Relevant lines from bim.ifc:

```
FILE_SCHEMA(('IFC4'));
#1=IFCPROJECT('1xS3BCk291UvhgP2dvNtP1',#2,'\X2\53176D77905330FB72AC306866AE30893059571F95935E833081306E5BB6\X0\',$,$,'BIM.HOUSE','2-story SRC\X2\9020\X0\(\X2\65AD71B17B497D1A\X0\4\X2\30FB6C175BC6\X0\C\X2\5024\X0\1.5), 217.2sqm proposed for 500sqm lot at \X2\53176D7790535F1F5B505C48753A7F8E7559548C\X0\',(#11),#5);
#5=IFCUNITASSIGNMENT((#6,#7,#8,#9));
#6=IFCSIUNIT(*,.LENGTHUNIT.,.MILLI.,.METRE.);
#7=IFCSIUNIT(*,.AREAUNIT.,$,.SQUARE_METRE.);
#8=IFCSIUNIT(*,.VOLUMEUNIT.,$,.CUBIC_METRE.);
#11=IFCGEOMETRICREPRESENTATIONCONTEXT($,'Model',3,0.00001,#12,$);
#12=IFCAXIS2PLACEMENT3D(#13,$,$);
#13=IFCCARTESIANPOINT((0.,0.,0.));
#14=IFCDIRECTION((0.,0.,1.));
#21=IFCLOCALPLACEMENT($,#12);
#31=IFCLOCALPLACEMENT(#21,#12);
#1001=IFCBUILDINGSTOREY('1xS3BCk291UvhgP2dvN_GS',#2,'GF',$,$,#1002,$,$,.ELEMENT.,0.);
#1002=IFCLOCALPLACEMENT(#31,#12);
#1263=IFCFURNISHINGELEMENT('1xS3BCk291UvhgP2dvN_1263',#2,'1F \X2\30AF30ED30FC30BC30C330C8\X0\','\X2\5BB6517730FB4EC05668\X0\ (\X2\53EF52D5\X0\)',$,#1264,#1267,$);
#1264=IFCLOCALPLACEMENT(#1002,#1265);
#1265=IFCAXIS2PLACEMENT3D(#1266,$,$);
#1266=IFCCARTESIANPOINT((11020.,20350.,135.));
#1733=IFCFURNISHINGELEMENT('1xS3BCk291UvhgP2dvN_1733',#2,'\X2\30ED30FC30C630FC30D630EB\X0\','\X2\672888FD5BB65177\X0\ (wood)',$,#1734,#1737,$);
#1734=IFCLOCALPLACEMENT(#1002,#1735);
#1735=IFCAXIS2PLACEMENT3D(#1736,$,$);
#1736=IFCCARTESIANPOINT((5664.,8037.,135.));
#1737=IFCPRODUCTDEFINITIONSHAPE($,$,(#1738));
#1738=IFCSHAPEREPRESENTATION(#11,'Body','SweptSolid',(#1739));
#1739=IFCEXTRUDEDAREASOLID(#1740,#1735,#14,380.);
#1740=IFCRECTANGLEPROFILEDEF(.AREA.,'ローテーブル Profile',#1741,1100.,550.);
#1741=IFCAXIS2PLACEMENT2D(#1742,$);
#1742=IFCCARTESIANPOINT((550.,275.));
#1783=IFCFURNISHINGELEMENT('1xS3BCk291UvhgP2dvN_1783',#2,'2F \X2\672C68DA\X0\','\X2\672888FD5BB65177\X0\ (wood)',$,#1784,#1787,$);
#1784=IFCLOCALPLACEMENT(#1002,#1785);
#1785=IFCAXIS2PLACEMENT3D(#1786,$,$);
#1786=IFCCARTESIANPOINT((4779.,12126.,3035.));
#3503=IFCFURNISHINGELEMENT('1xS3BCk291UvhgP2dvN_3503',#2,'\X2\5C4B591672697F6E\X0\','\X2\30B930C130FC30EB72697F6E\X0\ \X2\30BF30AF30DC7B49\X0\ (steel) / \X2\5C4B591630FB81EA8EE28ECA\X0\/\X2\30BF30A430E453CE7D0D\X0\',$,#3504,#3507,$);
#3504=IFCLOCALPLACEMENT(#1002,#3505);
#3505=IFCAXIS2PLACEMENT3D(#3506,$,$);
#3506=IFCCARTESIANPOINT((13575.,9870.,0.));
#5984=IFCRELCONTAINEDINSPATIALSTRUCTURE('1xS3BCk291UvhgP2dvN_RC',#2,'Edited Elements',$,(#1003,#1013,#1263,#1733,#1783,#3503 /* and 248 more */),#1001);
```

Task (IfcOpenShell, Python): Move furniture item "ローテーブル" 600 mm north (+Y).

```python
import ifcopenshell
import ifcopenshell.api.geometry
import ifcopenshell.util.placement

model = ifcopenshell.open("bim.ifc")

item = model.by_guid("1xS3BCk291UvhgP2dvN_1733")
matrix = ifcopenshell.util.placement.get_local_placement(item.ObjectPlacement)
matrix[1, 3] += 600.0
ifcopenshell.api.geometry.edit_object_placement(model, product=item, matrix=matrix, is_si=False)

print(ifcopenshell.util.placement.get_local_placement(item.ObjectPlacement).round(3) + 0.0)

model.write("bim_updated.ifc")
```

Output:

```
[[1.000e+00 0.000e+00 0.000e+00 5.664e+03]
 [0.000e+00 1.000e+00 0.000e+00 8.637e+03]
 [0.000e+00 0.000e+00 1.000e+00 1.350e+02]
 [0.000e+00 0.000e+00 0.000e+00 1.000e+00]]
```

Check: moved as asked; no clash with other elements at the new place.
